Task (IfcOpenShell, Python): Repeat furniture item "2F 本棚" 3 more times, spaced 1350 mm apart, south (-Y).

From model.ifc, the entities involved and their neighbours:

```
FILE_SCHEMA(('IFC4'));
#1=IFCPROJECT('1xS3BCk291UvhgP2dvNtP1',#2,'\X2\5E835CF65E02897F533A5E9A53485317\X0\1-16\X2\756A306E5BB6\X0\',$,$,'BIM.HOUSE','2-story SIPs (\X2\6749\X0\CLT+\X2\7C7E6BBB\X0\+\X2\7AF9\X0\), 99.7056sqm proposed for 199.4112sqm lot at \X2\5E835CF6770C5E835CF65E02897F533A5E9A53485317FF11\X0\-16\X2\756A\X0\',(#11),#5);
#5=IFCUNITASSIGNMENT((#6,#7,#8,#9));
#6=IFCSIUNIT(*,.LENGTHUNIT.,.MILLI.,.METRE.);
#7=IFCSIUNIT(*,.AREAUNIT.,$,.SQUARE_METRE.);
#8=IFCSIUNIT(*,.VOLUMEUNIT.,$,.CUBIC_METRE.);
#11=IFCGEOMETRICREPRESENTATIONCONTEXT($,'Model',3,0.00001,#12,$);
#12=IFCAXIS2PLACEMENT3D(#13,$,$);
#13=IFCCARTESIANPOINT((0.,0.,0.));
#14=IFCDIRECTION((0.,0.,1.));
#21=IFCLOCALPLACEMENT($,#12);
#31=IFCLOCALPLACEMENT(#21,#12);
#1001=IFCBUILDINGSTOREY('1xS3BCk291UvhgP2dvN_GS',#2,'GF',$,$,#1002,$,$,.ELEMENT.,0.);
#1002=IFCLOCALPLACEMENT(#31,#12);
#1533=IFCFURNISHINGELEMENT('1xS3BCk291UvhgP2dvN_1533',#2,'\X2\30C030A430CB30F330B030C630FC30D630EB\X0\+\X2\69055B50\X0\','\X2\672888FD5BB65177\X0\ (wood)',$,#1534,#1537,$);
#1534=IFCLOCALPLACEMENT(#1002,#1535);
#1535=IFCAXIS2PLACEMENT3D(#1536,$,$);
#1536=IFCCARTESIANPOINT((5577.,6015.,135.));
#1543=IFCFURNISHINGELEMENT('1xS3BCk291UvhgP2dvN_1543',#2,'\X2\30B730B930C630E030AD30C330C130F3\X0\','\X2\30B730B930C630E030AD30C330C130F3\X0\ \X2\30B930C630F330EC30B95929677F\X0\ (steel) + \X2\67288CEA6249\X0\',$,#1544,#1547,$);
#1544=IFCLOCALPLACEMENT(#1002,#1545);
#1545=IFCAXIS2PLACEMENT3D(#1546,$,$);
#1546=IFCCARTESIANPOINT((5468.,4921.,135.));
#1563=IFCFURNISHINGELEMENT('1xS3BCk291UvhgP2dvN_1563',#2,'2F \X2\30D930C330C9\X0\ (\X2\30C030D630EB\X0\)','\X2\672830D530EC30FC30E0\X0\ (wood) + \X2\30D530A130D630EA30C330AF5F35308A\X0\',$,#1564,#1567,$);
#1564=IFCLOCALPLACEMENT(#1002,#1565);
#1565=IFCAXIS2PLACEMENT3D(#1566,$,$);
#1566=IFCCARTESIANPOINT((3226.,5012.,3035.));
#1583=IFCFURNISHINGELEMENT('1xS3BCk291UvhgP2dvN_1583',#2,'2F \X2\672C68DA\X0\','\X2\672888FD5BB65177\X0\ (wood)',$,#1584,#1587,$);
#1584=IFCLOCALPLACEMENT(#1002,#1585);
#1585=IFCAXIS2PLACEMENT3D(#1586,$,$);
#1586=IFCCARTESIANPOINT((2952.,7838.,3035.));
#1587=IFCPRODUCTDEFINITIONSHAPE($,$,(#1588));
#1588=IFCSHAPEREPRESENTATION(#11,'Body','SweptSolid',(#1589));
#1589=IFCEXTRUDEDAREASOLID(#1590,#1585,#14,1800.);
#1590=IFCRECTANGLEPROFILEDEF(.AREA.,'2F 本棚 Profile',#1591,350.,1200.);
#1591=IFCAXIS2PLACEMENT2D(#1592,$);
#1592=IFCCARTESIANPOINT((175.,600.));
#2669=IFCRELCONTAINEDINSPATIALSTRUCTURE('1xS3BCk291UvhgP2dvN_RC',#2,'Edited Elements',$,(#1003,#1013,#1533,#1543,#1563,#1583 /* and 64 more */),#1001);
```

```python
import numpy as np
import ifcopenshell
import ifcopenshell.api.geometry
import ifcopenshell.api.root
import ifcopenshell.util.element
import ifcopenshell.util.placement
import ifcopenshell.util.unit

model = ifcopenshell.open("model.ifc")
unit_scale = ifcopenshell.util.unit.calculate_unit_scale(model)


def reuse_history(source, copy):
    """copy_class also copies each property set's owner history, people and application; keep the originals."""
    for rel in copy.IsDefinedBy:
        if rel.is_a("IfcRelDefinesByProperties") and (history := rel.RelatingPropertyDefinition.OwnerHistory):
            rel.RelatingPropertyDefinition.OwnerHistory = source.OwnerHistory
            ifcopenshell.util.element.remove_deep2(model, history)


source = model.by_guid("1xS3BCk291UvhgP2dvN_1583")
base = ifcopenshell.util.placement.get_local_placement(source.ObjectPlacement)
step = np.array([0.0, -1.0, 0.0]) * 1.35 / unit_scale

for i in range(1, 4):
    copy = ifcopenshell.api.root.copy_class(model, product=source)
    copy.Representation = ifcopenshell.util.element.copy_deep(
        model, source.Representation, exclude=["IfcGeometricRepresentationContext", "IfcRepresentationMap"]
    )
    reuse_history(source, copy)
    matrix = base.copy()
    matrix[:3, 3] += i * step
    print("added at", matrix[:3, 3].round(3) + 0.0)
    ifcopenshell.api.geometry.edit_object_placement(model, product=copy, matrix=matrix, is_si=False)

model.write("model_v2.ifc")
```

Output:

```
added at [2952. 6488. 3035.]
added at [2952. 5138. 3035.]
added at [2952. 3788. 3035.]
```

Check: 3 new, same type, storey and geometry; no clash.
